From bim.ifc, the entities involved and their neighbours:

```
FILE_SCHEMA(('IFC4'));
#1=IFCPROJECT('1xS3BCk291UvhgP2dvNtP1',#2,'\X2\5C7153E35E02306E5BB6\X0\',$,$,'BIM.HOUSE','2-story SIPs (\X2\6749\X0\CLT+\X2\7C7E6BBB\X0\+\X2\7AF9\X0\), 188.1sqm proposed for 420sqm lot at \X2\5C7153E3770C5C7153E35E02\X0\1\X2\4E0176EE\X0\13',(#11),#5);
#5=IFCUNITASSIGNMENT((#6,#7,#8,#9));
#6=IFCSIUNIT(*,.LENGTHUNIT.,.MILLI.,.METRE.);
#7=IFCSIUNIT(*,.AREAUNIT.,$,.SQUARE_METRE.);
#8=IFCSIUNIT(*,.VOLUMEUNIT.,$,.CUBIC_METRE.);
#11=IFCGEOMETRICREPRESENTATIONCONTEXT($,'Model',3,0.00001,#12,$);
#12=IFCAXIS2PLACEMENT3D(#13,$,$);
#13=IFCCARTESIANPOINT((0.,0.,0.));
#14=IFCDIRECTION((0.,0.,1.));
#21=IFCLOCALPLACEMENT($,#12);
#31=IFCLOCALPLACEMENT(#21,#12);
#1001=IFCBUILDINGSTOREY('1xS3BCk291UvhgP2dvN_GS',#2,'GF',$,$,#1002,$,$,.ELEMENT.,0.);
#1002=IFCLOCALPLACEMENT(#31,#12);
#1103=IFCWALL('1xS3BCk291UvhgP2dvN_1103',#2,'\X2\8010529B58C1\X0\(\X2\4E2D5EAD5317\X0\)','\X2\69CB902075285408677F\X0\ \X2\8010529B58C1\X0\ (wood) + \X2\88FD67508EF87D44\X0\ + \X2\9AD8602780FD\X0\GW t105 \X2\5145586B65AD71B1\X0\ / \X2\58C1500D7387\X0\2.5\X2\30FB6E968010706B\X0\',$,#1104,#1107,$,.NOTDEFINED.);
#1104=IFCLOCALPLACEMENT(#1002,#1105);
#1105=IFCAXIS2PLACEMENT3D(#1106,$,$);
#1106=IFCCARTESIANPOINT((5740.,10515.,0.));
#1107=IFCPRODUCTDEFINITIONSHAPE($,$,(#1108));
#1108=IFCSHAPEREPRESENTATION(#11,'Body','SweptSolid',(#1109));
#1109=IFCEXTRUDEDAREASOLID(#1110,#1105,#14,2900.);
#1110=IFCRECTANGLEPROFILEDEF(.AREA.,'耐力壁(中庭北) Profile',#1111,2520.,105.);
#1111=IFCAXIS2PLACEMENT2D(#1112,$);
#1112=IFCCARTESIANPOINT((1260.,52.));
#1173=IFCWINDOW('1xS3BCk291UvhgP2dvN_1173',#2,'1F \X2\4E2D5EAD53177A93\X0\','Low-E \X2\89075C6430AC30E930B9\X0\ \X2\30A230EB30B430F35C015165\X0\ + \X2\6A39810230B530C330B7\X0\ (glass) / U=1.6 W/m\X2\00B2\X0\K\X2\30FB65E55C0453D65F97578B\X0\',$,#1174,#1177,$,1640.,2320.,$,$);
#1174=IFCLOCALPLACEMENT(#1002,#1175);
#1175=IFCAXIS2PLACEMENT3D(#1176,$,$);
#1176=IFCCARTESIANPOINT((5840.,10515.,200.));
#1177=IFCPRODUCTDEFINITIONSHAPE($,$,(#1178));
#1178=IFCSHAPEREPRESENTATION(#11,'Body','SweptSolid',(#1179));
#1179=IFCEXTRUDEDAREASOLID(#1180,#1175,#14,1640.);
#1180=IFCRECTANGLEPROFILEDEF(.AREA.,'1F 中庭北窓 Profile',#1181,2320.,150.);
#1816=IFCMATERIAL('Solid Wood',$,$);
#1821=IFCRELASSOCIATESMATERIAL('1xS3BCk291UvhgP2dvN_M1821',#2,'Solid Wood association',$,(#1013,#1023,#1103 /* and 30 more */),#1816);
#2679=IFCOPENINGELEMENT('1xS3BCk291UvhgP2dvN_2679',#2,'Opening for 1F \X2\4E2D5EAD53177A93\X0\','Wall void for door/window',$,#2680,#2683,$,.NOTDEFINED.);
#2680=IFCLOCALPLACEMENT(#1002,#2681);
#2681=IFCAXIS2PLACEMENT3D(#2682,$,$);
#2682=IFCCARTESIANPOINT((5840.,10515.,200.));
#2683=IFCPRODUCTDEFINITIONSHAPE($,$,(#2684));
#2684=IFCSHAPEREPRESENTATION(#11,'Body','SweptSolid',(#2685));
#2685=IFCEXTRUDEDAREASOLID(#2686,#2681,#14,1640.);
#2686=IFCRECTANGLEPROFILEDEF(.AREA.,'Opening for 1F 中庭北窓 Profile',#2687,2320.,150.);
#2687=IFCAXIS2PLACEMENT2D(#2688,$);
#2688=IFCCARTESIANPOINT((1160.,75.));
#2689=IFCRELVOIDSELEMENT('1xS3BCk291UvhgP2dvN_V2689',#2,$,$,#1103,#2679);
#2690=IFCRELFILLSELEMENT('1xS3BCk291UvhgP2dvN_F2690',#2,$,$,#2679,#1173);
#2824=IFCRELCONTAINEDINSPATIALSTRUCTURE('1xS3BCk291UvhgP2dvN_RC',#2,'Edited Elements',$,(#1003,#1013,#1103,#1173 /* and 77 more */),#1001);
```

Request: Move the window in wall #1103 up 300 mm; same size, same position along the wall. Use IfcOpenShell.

```python
import numpy as np
import ifcopenshell
import ifcopenshell.api.geometry
import ifcopenshell.util.placement
import ifcopenshell.util.unit

model = ifcopenshell.open("bim.ifc")
unit_scale = ifcopenshell.util.unit.calculate_unit_scale(model)

window = model.by_guid("1xS3BCk291UvhgP2dvN_1173")
opening = window.FillsVoids[0].RelatingOpeningElement
dz = 0.3 / unit_scale

shift = np.array([0.0, 0.0, dz])
# The window is not placed relative to its opening, so move both.
for product in (opening, window):
    matrix = ifcopenshell.util.placement.get_local_placement(product.ObjectPlacement)
    matrix[:3, 3] += shift
    ifcopenshell.api.geometry.edit_object_placement(model, product=product, matrix=matrix, is_si=False)

print(f"moved by {dz * unit_scale:+.3f} m")

model.write("bim_v2.ifc")
```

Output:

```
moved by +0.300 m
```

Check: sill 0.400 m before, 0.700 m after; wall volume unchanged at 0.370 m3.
